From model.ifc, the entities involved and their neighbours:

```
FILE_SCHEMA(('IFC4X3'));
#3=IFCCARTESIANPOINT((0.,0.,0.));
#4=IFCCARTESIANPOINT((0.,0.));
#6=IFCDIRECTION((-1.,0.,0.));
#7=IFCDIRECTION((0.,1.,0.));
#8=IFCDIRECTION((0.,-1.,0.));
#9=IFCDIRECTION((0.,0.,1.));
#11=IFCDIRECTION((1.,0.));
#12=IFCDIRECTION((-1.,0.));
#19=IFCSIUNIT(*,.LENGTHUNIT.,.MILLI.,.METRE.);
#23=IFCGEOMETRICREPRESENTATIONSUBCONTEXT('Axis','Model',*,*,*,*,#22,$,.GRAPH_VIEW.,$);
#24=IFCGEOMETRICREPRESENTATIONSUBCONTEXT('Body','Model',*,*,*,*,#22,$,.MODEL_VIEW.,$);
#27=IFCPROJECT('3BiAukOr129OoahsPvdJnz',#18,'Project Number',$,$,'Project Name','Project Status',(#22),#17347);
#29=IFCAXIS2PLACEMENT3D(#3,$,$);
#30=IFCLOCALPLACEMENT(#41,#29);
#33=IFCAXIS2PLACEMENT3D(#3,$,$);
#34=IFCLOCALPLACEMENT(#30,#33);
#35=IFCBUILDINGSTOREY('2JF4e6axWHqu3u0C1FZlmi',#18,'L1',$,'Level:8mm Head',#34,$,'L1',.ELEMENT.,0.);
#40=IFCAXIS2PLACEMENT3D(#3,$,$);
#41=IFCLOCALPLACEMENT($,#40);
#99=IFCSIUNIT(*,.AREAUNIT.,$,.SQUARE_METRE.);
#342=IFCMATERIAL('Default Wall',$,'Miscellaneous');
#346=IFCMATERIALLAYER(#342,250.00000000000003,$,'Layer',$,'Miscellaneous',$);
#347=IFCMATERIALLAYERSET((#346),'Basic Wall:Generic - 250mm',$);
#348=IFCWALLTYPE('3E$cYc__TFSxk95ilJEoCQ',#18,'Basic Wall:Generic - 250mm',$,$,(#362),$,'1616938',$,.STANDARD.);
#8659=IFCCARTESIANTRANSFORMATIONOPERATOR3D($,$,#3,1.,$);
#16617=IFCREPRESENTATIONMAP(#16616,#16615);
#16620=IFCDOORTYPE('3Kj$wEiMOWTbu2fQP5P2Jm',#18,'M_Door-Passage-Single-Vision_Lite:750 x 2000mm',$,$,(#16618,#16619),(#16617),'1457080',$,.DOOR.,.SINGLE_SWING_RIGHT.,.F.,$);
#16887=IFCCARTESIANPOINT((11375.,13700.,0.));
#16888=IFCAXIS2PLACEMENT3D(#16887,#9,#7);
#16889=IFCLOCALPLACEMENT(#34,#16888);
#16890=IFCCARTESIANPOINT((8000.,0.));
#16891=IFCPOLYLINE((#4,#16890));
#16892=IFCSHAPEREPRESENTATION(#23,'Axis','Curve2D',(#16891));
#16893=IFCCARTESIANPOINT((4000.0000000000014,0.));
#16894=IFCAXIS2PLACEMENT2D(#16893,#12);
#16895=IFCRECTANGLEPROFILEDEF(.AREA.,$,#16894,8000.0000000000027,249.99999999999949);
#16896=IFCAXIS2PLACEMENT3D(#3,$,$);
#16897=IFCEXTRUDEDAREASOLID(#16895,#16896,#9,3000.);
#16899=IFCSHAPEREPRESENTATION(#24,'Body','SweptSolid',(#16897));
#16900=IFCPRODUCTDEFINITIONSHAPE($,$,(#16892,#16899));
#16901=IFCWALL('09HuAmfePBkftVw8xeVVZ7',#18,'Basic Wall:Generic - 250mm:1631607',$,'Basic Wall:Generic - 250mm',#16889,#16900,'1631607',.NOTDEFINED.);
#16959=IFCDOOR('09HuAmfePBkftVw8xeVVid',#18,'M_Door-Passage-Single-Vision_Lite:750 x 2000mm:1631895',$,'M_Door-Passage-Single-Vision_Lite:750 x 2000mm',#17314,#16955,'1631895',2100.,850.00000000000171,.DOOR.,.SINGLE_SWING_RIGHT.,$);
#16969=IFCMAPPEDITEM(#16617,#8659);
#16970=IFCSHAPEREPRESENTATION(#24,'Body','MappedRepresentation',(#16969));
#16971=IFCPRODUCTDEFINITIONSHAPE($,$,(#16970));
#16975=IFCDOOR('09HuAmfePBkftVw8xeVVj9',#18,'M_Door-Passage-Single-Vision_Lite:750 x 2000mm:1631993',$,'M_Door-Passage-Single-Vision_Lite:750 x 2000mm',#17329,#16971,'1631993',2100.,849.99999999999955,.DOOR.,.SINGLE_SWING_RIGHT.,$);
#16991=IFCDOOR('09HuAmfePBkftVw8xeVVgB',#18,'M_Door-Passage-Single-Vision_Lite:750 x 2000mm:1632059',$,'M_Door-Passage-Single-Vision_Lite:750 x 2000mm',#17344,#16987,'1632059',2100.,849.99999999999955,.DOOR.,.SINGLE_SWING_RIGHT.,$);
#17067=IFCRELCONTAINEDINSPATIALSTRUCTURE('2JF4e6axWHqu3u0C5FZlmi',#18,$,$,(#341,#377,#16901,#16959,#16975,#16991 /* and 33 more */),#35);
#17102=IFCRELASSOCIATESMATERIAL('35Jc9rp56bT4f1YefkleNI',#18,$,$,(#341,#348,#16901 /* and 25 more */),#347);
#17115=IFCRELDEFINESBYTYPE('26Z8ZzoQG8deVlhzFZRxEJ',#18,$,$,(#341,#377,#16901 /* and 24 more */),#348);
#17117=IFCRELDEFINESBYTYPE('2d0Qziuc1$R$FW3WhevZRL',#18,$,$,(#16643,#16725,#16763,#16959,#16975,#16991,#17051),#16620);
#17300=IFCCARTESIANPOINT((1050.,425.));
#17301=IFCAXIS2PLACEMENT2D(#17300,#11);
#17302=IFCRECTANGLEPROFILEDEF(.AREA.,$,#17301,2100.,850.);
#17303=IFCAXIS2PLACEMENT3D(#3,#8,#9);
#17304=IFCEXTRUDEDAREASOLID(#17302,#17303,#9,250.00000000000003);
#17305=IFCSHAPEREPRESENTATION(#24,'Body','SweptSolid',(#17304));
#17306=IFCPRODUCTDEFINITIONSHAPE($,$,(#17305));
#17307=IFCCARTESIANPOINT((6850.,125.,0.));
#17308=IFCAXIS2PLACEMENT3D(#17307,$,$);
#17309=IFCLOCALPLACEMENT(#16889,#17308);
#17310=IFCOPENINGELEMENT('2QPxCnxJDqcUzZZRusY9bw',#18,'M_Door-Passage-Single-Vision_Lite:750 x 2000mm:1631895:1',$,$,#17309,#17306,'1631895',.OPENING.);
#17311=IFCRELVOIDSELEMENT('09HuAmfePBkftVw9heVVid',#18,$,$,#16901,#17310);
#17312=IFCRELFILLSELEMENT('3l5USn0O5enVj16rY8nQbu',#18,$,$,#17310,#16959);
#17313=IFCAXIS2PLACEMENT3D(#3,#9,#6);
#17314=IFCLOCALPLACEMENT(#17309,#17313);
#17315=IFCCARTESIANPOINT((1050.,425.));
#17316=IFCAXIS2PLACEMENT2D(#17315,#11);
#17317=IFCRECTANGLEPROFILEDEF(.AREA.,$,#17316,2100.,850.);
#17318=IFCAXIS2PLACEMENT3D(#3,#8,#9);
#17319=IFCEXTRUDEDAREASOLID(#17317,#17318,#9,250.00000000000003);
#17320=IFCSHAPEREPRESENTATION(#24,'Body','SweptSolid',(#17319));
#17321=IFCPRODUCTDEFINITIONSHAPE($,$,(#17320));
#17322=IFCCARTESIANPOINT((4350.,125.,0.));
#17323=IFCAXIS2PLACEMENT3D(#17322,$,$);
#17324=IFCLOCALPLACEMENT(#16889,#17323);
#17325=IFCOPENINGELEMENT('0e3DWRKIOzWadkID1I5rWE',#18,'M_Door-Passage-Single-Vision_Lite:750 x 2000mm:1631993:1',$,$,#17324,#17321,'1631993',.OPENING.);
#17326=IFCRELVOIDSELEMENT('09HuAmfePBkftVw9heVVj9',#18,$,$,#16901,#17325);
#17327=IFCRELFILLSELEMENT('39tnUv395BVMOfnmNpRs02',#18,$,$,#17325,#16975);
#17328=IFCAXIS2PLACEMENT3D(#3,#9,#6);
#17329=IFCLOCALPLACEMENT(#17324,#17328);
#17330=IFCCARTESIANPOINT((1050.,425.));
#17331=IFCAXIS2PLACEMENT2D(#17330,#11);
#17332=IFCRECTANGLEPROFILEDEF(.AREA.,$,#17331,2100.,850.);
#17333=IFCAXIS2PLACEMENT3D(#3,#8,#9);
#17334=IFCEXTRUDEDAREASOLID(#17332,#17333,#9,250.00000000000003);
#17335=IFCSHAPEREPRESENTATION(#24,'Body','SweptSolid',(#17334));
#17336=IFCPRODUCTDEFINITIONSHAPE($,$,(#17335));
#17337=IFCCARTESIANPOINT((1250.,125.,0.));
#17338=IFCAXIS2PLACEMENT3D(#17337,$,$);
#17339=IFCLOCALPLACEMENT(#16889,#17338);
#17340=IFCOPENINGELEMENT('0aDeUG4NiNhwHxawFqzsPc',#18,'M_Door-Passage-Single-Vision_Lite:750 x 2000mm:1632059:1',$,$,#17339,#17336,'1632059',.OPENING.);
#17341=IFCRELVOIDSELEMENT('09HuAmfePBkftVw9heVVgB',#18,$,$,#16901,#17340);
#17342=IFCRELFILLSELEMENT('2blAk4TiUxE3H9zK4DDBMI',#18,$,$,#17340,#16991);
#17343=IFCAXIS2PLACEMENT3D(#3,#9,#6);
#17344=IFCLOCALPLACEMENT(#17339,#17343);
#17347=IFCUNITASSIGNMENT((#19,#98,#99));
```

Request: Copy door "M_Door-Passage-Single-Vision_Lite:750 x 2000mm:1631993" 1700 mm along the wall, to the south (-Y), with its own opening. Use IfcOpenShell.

```python
import ifcopenshell
import ifcopenshell.api.feature
import ifcopenshell.api.geometry
import ifcopenshell.api.root
import ifcopenshell.geom
import ifcopenshell.util.element
import ifcopenshell.util.placement
import ifcopenshell.util.shape

model = ifcopenshell.open("model.ifc")
settings = ifcopenshell.geom.settings()


def volume(element):
    """Net volume in cubic metres, openings subtracted."""
    shape = ifcopenshell.geom.create_shape(settings, element)
    return ifcopenshell.util.shape.get_volume(shape.geometry)


def reuse_history(source, copy):
    """copy_class also copies each property set's owner history, people and application; keep the originals."""
    for rel in copy.IsDefinedBy:
        if rel.is_a("IfcRelDefinesByProperties") and (history := rel.RelatingPropertyDefinition.OwnerHistory):
            rel.RelatingPropertyDefinition.OwnerHistory = source.OwnerHistory
            ifcopenshell.util.element.remove_deep2(model, history)


door = model.by_id(16975)
opening = door.FillsVoids[0].RelatingOpeningElement
wall = opening.VoidsElements[0].RelatingBuildingElement
before = volume(wall)
shift = ifcopenshell.util.placement.get_local_placement(wall.ObjectPlacement)[:3, 0] * -1700.0

# copy_class copies the void relationship, type, container and properties, but no geometry.
new_opening = ifcopenshell.api.root.copy_class(model, product=opening)
new_opening.Representation = ifcopenshell.util.element.copy_deep(
    model, opening.Representation, exclude=["IfcGeometricRepresentationContext", "IfcRepresentationMap"]
)
new_opening.Name = "M_Door-Passage-Single-Vision_Lite:750 x 2000mm"
new_opening.Tag = None
new_door = ifcopenshell.api.root.copy_class(model, product=door)
new_door.Representation = ifcopenshell.util.element.copy_deep(
    model, door.Representation, exclude=["IfcGeometricRepresentationContext", "IfcRepresentationMap"]
)
new_door.Name = "M_Door-Passage-Single-Vision_Lite:750 x 2000mm"
new_door.Tag = None
reuse_history(door, new_door)
ifcopenshell.api.feature.add_filling(model, opening=new_opening, element=new_door)

for old, new in ((opening, new_opening), (door, new_door)):
    matrix = ifcopenshell.util.placement.get_local_placement(old.ObjectPlacement)
    matrix[:3, 3] += shift
    ifcopenshell.api.geometry.edit_object_placement(model, product=new, matrix=matrix, is_si=False)

after = volume(wall)

print(f"wall volume {before:.3f} -> {after:.3f} m3")

model.write("model_rev.ifc")
```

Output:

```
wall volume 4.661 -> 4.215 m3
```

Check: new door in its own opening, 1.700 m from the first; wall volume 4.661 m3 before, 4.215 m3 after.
